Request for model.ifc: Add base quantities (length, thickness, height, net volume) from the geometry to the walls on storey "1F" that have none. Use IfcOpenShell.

First a look at what the model holds.

```python
import ifcopenshell
import ifcopenshell.util.element
import ifcopenshell.util.unit

model = ifcopenshell.open("model.ifc")
print(model.schema)
for unit_type in ("LENGTHUNIT", "AREAUNIT", "VOLUMEUNIT"):
    print(unit_type, ifcopenshell.util.unit.calculate_unit_scale(model, unit_type))
storey = next(s for s in model.by_type("IfcBuildingStorey") if s.Name == "1F")
walls = [e for e in ifcopenshell.util.element.get_decomposition(storey) if e.is_a("IfcWall")]
for e in sorted(walls, key=lambda e: e.id()):
    print(e.id(), e.is_a(), e.Name, list(ifcopenshell.util.element.get_psets(e, qtos_only=True)), sep=" | ")
```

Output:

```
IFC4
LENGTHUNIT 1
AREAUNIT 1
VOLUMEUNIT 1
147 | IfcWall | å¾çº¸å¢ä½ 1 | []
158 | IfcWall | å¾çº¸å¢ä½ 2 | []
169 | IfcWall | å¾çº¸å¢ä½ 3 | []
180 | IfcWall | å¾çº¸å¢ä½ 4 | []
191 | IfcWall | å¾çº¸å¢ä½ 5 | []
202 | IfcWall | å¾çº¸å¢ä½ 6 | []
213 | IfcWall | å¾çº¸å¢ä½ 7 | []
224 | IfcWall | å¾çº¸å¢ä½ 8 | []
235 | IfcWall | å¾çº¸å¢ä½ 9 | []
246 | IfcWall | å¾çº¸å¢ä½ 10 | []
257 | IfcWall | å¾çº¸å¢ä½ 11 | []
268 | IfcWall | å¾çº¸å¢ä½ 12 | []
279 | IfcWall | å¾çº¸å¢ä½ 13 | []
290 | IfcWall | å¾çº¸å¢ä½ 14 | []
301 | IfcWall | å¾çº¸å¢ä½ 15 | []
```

```python
import ifcopenshell
import ifcopenshell.api.pset
import ifcopenshell.geom
import ifcopenshell.util.element
import ifcopenshell.util.shape
import ifcopenshell.util.unit

model = ifcopenshell.open("model.ifc")
unit_scale = ifcopenshell.util.unit.calculate_unit_scale(model)
volume_scale = ifcopenshell.util.unit.calculate_unit_scale(model, "VOLUMEUNIT")
settings = ifcopenshell.geom.settings()

storey = next(s for s in model.by_type("IfcBuildingStorey") if s.Name == "1F")
walls = [e for e in ifcopenshell.util.element.get_decomposition(storey) if e.is_a("IfcWall")]

for e in sorted(walls, key=lambda e: e.id()):
    if ifcopenshell.util.element.get_psets(e, qtos_only=True, should_inherit=False):
        continue
    # Geometry comes back in metres, in the element's own axes.
    shape = ifcopenshell.geom.create_shape(settings, e)
    values = {
        "Length": ifcopenshell.util.shape.get_x(shape.geometry) / unit_scale,
        "Width": ifcopenshell.util.shape.get_y(shape.geometry) / unit_scale,
        "Height": ifcopenshell.util.shape.get_z(shape.geometry) / unit_scale,
        "NetVolume": ifcopenshell.util.shape.get_volume(shape.geometry) / volume_scale,
    }
    qto = ifcopenshell.api.pset.add_qto(model, product=e, name="Qto_WallBaseQuantities")
    ifcopenshell.api.pset.edit_qto(model, qto=qto, properties=values)
    print(e.id(), {k: round(v, 3) for k, v in values.items()})

model.write("model_rev.ifc")
```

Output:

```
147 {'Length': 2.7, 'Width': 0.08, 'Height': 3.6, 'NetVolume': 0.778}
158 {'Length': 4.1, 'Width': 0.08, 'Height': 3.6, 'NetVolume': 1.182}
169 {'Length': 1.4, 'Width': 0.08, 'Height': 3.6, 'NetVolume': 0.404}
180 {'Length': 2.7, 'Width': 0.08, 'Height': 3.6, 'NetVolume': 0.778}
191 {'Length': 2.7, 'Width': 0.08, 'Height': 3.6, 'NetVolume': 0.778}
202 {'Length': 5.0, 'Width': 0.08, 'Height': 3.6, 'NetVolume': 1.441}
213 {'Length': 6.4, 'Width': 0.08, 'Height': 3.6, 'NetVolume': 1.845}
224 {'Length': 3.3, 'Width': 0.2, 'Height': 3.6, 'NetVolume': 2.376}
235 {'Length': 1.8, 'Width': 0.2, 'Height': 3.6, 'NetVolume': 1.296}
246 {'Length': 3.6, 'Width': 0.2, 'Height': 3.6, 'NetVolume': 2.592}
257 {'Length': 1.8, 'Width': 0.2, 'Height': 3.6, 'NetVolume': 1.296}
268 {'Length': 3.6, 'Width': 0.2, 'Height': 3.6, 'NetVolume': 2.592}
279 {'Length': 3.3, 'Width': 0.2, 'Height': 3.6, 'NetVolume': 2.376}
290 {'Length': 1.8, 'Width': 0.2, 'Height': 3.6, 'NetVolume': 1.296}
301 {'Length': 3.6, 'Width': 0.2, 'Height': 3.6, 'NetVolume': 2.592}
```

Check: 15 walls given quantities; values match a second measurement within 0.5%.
